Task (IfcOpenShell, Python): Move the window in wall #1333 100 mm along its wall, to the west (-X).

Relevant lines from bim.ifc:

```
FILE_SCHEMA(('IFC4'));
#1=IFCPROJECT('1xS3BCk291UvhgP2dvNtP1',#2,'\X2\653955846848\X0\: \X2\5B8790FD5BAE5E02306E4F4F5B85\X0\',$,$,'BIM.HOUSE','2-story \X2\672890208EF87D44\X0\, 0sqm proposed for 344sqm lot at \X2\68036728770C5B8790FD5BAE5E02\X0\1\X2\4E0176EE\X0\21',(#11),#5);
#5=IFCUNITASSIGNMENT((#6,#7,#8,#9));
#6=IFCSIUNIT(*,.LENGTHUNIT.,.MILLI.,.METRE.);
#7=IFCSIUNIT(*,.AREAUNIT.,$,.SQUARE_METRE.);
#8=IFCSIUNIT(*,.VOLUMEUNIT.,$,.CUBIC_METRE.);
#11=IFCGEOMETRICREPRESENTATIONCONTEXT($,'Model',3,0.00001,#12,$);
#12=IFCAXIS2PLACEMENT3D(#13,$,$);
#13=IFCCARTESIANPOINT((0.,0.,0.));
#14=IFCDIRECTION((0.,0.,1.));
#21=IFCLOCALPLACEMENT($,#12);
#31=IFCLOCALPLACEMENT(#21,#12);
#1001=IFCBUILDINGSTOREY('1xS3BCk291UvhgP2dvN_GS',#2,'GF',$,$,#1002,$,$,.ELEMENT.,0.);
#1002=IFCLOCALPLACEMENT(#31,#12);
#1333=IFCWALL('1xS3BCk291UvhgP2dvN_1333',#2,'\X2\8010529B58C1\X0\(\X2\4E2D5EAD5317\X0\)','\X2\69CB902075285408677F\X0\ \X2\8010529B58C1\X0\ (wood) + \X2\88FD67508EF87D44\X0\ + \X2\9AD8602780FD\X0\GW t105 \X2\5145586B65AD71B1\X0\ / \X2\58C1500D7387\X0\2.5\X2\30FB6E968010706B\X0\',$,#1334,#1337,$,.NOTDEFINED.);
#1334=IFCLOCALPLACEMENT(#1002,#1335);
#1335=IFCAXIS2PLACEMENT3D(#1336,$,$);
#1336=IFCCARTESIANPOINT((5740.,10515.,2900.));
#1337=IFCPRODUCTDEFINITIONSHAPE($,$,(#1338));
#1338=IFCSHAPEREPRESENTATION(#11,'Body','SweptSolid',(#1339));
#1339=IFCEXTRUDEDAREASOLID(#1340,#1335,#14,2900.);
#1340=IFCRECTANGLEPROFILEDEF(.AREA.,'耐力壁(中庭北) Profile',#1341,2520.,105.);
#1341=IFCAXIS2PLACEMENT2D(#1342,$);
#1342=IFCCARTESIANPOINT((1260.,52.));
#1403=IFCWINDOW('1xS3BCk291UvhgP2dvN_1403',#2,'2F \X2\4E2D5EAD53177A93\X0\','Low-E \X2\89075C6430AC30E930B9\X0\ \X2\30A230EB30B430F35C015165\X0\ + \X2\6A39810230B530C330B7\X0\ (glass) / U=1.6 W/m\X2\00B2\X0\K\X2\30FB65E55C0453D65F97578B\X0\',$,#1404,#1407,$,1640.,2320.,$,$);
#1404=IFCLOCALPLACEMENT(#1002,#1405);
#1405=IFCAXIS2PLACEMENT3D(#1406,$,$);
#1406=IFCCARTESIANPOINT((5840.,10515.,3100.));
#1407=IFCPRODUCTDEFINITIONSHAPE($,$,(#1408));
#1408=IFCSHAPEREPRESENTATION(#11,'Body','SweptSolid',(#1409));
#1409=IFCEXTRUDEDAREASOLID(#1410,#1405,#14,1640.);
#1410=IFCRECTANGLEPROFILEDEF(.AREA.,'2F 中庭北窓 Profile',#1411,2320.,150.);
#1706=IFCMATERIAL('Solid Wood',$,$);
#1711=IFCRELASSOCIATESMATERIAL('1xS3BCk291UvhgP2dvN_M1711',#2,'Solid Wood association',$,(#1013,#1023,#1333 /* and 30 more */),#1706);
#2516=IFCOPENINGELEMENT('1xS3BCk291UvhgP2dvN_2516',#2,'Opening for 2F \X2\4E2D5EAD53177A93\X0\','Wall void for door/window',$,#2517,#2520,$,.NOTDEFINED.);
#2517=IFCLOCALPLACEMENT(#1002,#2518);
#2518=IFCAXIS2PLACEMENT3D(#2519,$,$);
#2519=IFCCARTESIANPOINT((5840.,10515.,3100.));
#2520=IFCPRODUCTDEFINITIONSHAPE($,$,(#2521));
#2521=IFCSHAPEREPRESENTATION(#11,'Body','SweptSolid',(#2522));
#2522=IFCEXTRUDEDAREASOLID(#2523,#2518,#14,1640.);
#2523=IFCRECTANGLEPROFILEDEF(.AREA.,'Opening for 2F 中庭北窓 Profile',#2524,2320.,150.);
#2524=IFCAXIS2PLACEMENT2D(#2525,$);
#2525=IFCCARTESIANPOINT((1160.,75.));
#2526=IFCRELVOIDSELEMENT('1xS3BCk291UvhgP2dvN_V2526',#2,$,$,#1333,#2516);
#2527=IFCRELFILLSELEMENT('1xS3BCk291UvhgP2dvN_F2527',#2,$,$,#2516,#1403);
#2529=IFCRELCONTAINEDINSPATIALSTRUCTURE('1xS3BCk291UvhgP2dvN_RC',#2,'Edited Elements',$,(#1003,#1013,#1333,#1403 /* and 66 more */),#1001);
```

```python
import ifcopenshell
import ifcopenshell.api.geometry
import ifcopenshell.util.placement
import ifcopenshell.util.unit

model = ifcopenshell.open("bim.ifc")
unit_scale = ifcopenshell.util.unit.calculate_unit_scale(model)

window = model.by_id(1403)
opening = window.FillsVoids[0].RelatingOpeningElement
wall = opening.VoidsElements[0].RelatingBuildingElement

wall_matrix = ifcopenshell.util.placement.get_local_placement(wall.ObjectPlacement)
shift = wall_matrix[:3, 0] * -0.1 / unit_scale
before = ifcopenshell.util.placement.get_local_placement(window.ObjectPlacement)[:3, 3].copy()

# The window is not placed relative to its opening, so move both.
for product in (opening, window):
    matrix = ifcopenshell.util.placement.get_local_placement(product.ObjectPlacement)
    matrix[:3, 3] += shift
    ifcopenshell.api.geometry.edit_object_placement(model, product=product, matrix=matrix, is_si=False)

after = ifcopenshell.util.placement.get_local_placement(window.ObjectPlacement)[:3, 3]
print("window moved by", (after - before).round(3) + 0.0)

model.write("bim_v2.ifc")
```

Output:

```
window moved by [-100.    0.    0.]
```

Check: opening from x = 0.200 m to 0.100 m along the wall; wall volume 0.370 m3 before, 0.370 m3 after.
